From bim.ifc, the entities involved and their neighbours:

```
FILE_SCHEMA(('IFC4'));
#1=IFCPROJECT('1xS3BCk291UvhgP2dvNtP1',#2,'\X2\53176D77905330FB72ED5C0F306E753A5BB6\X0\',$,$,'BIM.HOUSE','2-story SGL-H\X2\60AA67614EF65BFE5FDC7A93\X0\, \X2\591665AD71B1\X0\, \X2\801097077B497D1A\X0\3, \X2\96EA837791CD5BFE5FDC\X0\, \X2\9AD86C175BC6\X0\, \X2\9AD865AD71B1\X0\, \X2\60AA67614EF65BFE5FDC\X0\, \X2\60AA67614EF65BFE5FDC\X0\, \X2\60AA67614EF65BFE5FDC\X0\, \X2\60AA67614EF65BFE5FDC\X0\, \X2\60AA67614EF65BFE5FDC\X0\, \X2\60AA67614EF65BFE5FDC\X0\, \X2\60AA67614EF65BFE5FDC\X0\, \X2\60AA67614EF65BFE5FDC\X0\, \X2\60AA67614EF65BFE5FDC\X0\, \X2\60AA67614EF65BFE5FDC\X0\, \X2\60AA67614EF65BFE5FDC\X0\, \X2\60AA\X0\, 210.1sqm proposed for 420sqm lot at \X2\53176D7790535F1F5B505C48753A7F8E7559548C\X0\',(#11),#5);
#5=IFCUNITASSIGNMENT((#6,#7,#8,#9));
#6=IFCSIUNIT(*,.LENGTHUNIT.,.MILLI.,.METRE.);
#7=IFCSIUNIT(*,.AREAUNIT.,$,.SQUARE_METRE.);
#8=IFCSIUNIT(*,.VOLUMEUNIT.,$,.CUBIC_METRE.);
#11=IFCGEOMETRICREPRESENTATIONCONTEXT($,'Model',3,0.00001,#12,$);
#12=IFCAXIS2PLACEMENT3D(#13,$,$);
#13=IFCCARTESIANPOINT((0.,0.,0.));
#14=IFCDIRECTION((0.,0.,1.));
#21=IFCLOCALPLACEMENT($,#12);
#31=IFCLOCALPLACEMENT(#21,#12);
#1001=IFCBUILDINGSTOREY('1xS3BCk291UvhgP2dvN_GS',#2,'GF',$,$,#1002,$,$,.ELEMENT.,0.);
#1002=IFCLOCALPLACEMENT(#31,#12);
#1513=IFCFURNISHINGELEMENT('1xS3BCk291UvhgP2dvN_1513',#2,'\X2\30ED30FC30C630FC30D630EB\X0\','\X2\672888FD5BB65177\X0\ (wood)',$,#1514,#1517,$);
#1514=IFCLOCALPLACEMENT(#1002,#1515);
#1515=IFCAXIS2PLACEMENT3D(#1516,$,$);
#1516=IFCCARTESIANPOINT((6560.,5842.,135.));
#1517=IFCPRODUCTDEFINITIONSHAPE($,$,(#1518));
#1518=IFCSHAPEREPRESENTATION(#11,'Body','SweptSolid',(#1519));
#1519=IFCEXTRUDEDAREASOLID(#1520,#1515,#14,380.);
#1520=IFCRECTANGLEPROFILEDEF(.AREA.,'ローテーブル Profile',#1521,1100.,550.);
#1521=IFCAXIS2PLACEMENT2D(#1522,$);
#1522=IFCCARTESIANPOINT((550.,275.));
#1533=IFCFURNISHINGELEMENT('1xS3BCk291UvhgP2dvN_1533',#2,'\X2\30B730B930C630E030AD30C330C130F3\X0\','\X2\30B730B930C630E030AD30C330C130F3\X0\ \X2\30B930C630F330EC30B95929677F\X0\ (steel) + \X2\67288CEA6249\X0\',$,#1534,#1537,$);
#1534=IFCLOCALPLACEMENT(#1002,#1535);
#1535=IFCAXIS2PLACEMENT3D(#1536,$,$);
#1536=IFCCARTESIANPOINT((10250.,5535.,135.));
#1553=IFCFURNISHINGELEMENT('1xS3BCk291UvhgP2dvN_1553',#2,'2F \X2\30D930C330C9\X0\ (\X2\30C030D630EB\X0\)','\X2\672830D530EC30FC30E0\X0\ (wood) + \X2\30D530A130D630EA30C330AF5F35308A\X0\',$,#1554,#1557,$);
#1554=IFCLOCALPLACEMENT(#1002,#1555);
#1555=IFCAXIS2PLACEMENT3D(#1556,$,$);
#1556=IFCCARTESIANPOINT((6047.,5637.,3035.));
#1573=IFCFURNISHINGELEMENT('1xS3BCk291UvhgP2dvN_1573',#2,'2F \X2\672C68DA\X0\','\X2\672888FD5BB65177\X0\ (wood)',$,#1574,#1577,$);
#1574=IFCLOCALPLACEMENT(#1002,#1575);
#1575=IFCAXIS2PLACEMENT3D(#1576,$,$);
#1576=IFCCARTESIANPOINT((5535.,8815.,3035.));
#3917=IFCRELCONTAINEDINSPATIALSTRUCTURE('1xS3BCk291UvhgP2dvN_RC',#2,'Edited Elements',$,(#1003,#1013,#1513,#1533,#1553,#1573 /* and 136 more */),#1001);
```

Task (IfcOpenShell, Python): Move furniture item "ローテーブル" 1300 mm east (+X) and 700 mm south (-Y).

```python
import ifcopenshell
import ifcopenshell.api.geometry
import ifcopenshell.util.placement

model = ifcopenshell.open("bim.ifc")

item = model.by_id(1513)
matrix = ifcopenshell.util.placement.get_local_placement(item.ObjectPlacement)
matrix[0, 3] += 1300.0
matrix[1, 3] -= 700.0
ifcopenshell.api.geometry.edit_object_placement(model, product=item, matrix=matrix, is_si=False)

print(ifcopenshell.util.placement.get_local_placement(item.ObjectPlacement).round(3) + 0.0)

model.write("bim-out.ifc")
```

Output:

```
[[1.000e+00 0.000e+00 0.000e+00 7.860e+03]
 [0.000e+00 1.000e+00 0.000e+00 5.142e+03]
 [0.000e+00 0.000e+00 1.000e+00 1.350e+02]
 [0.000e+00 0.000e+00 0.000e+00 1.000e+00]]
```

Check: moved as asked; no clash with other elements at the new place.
